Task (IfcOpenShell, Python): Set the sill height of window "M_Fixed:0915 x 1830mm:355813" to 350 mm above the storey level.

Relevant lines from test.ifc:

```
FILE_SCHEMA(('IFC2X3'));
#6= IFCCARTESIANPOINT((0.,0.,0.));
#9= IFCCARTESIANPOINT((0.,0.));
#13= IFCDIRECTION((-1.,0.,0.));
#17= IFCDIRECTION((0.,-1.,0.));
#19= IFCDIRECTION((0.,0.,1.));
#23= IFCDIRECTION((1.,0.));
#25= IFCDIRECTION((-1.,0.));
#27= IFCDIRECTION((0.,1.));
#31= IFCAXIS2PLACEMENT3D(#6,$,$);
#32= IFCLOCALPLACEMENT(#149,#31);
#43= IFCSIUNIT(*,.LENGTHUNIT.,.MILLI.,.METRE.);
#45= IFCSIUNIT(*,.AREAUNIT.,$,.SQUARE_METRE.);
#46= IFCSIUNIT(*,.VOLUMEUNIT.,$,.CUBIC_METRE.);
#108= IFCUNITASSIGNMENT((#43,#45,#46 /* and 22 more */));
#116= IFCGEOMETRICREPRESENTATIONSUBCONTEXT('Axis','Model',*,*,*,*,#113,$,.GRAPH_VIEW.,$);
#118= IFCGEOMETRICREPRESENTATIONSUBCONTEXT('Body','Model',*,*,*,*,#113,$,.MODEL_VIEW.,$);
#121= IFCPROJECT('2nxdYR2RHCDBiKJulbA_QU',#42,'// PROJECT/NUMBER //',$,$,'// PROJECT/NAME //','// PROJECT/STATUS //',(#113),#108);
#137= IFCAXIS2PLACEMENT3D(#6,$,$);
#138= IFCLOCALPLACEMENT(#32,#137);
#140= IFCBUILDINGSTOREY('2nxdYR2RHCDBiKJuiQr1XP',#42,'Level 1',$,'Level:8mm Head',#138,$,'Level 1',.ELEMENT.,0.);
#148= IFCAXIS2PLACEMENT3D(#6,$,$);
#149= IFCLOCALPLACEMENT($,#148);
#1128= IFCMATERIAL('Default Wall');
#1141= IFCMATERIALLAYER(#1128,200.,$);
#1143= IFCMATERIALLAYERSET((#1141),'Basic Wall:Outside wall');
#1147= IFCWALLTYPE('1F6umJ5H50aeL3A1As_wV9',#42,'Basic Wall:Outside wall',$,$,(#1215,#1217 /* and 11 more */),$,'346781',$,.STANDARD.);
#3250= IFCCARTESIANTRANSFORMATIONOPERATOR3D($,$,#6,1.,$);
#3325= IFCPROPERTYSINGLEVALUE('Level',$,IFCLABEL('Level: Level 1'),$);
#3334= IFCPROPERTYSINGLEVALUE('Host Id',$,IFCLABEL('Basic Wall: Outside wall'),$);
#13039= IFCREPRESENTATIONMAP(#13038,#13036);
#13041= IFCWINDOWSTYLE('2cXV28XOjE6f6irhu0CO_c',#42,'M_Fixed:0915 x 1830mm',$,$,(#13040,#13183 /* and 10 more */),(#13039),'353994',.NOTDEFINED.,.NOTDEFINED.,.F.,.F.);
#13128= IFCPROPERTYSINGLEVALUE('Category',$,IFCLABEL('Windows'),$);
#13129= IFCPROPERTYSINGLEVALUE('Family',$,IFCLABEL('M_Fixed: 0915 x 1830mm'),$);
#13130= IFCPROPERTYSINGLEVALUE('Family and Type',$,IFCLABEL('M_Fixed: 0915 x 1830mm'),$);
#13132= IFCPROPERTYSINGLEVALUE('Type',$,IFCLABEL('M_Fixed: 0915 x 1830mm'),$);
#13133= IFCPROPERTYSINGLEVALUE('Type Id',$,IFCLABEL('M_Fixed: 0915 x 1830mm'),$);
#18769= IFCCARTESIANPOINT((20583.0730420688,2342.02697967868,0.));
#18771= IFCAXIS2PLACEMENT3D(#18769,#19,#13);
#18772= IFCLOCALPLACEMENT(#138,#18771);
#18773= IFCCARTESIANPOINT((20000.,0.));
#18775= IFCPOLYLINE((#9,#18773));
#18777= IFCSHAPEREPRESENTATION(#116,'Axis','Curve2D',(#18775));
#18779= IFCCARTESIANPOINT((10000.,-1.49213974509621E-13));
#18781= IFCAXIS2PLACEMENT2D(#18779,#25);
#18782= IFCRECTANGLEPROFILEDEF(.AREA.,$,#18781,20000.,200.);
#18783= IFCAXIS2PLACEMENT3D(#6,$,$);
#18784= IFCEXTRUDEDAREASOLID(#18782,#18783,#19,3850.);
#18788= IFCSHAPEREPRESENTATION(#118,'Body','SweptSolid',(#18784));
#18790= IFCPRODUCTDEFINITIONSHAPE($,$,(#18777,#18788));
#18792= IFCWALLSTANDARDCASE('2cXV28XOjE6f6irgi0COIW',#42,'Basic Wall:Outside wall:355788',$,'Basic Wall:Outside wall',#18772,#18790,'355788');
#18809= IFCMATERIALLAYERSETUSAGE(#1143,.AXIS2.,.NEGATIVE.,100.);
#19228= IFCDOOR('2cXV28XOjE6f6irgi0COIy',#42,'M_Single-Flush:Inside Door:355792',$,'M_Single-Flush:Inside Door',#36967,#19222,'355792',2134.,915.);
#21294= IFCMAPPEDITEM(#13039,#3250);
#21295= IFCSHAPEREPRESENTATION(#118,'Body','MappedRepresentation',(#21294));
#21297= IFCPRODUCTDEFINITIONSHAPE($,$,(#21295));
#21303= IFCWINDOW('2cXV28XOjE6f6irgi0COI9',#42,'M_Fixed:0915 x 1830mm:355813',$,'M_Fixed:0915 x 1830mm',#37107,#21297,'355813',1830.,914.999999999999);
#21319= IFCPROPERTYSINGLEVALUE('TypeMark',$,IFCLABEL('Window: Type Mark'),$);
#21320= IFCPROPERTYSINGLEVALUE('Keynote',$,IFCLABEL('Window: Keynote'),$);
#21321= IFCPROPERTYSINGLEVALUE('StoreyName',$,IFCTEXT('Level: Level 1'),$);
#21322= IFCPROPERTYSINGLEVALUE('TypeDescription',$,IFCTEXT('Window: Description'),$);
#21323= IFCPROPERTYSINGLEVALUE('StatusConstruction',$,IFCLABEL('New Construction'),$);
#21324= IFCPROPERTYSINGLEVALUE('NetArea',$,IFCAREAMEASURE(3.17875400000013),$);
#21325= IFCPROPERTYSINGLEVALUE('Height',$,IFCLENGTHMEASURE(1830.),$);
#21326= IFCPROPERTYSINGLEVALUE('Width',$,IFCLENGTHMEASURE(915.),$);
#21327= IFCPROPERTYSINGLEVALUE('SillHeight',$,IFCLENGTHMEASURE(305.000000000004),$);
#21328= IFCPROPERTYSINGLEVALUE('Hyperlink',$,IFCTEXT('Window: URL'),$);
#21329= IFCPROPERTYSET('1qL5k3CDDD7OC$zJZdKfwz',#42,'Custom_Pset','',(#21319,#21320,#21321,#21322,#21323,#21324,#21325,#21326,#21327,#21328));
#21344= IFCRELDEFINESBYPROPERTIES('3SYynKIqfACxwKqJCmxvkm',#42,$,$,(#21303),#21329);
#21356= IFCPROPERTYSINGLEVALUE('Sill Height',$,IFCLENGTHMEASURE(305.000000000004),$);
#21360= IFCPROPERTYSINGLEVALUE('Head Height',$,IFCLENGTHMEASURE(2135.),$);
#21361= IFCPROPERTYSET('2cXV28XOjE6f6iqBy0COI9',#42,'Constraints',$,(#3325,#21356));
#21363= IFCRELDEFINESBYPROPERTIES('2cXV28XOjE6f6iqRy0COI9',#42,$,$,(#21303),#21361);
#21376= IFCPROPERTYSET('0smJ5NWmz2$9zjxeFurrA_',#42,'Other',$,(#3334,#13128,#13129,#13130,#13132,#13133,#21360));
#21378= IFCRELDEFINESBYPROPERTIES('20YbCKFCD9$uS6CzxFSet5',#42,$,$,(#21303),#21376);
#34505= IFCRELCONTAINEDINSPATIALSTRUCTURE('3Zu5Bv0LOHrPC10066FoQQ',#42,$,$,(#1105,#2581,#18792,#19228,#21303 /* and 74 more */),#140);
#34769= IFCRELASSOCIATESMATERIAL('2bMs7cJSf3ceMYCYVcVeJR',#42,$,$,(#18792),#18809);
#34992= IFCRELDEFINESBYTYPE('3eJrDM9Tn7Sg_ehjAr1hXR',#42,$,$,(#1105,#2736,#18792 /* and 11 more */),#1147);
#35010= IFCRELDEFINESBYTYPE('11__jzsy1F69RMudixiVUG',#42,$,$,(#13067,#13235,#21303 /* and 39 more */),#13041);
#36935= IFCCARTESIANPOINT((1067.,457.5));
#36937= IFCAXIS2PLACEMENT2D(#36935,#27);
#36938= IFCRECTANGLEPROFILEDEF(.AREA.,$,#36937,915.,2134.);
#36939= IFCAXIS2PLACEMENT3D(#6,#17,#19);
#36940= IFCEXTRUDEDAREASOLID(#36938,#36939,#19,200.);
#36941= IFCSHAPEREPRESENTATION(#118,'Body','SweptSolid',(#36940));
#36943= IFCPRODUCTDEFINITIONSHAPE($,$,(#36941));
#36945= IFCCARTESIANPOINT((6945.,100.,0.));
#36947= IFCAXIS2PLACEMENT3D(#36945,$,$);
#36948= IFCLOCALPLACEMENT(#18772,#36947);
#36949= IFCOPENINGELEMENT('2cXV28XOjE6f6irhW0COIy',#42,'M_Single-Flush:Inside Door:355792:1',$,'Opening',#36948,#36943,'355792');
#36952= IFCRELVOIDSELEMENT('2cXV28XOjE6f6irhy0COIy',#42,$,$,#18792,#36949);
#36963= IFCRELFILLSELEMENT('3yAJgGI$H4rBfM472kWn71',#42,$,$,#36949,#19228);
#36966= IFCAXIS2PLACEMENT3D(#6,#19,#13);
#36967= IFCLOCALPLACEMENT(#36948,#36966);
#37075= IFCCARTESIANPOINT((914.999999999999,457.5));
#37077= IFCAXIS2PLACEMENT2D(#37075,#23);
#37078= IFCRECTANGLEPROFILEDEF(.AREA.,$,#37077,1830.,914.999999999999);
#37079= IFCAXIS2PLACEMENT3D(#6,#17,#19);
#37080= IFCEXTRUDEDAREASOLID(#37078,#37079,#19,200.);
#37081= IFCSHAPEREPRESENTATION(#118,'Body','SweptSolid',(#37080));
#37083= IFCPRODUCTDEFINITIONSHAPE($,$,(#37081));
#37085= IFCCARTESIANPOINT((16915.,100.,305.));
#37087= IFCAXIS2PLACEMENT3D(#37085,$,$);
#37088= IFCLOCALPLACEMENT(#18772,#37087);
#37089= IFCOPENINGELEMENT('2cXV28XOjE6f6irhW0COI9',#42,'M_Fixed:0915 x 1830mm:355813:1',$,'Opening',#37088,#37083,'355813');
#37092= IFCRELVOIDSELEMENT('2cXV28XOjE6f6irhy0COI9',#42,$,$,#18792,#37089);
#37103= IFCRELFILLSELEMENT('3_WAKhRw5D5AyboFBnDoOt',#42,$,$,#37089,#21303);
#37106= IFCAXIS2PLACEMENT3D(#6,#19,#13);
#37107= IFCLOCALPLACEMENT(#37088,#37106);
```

```python
import numpy as np
import ifcopenshell
import ifcopenshell.api.geometry
import ifcopenshell.api.pset
import ifcopenshell.geom
import ifcopenshell.util.element
import ifcopenshell.util.placement
import ifcopenshell.util.shape
import ifcopenshell.util.unit

model = ifcopenshell.open("test.ifc")
unit_scale = ifcopenshell.util.unit.calculate_unit_scale(model)

window = model.by_id(21303)
opening = window.FillsVoids[0].RelatingOpeningElement
storey = ifcopenshell.util.element.get_container(window, ifc_class="IfcBuildingStorey")
level = ifcopenshell.util.placement.get_local_placement(storey.ObjectPlacement)[2, 3]

# The opening's origin need not be at the sill, so measure its lowest point.
shape = ifcopenshell.geom.create_shape(ifcopenshell.geom.settings(), opening)
bottom = ifcopenshell.util.shape.get_shape_bottom_elevation(shape, shape.geometry) / unit_scale
dz = level + 0.35 / unit_scale - bottom

shift = np.array([0.0, 0.0, dz])
# The window is placed relative to its opening, so it follows when the opening moves.
matrix = ifcopenshell.util.placement.get_local_placement(opening.ObjectPlacement)
matrix[:3, 3] += shift
ifcopenshell.api.geometry.edit_object_placement(
    model, product=opening, matrix=matrix, is_si=False, should_transform_children=True
)

# Keep the stored heights in step.
pset = model.by_id(ifcopenshell.util.element.get_pset(window, "Custom_Pset", should_inherit=False)["id"])
ifcopenshell.api.pset.edit_pset(model, pset=pset, properties={
    "SillHeight": model.create_entity("IfcLengthMeasure", ifcopenshell.util.element.get_pset(window, "Constraints", "Sill Height") + dz),
})
pset = model.by_id(ifcopenshell.util.element.get_pset(window, "Constraints", should_inherit=False)["id"])
ifcopenshell.api.pset.edit_pset(model, pset=pset, properties={
    "Sill Height": model.create_entity("IfcLengthMeasure", ifcopenshell.util.element.get_pset(window, "Constraints", "Sill Height") + dz),
})
pset = model.by_id(ifcopenshell.util.element.get_pset(window, "Other", should_inherit=False)["id"])
ifcopenshell.api.pset.edit_pset(model, pset=pset, properties={
    "Head Height": model.create_entity("IfcLengthMeasure", ifcopenshell.util.element.get_pset(window, "Other", "Head Height") + dz),
})

print(f"moved by {dz * unit_scale:+.3f} m")

model.write("test-out.ifc")
```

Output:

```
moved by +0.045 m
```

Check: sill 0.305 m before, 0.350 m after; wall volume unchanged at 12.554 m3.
